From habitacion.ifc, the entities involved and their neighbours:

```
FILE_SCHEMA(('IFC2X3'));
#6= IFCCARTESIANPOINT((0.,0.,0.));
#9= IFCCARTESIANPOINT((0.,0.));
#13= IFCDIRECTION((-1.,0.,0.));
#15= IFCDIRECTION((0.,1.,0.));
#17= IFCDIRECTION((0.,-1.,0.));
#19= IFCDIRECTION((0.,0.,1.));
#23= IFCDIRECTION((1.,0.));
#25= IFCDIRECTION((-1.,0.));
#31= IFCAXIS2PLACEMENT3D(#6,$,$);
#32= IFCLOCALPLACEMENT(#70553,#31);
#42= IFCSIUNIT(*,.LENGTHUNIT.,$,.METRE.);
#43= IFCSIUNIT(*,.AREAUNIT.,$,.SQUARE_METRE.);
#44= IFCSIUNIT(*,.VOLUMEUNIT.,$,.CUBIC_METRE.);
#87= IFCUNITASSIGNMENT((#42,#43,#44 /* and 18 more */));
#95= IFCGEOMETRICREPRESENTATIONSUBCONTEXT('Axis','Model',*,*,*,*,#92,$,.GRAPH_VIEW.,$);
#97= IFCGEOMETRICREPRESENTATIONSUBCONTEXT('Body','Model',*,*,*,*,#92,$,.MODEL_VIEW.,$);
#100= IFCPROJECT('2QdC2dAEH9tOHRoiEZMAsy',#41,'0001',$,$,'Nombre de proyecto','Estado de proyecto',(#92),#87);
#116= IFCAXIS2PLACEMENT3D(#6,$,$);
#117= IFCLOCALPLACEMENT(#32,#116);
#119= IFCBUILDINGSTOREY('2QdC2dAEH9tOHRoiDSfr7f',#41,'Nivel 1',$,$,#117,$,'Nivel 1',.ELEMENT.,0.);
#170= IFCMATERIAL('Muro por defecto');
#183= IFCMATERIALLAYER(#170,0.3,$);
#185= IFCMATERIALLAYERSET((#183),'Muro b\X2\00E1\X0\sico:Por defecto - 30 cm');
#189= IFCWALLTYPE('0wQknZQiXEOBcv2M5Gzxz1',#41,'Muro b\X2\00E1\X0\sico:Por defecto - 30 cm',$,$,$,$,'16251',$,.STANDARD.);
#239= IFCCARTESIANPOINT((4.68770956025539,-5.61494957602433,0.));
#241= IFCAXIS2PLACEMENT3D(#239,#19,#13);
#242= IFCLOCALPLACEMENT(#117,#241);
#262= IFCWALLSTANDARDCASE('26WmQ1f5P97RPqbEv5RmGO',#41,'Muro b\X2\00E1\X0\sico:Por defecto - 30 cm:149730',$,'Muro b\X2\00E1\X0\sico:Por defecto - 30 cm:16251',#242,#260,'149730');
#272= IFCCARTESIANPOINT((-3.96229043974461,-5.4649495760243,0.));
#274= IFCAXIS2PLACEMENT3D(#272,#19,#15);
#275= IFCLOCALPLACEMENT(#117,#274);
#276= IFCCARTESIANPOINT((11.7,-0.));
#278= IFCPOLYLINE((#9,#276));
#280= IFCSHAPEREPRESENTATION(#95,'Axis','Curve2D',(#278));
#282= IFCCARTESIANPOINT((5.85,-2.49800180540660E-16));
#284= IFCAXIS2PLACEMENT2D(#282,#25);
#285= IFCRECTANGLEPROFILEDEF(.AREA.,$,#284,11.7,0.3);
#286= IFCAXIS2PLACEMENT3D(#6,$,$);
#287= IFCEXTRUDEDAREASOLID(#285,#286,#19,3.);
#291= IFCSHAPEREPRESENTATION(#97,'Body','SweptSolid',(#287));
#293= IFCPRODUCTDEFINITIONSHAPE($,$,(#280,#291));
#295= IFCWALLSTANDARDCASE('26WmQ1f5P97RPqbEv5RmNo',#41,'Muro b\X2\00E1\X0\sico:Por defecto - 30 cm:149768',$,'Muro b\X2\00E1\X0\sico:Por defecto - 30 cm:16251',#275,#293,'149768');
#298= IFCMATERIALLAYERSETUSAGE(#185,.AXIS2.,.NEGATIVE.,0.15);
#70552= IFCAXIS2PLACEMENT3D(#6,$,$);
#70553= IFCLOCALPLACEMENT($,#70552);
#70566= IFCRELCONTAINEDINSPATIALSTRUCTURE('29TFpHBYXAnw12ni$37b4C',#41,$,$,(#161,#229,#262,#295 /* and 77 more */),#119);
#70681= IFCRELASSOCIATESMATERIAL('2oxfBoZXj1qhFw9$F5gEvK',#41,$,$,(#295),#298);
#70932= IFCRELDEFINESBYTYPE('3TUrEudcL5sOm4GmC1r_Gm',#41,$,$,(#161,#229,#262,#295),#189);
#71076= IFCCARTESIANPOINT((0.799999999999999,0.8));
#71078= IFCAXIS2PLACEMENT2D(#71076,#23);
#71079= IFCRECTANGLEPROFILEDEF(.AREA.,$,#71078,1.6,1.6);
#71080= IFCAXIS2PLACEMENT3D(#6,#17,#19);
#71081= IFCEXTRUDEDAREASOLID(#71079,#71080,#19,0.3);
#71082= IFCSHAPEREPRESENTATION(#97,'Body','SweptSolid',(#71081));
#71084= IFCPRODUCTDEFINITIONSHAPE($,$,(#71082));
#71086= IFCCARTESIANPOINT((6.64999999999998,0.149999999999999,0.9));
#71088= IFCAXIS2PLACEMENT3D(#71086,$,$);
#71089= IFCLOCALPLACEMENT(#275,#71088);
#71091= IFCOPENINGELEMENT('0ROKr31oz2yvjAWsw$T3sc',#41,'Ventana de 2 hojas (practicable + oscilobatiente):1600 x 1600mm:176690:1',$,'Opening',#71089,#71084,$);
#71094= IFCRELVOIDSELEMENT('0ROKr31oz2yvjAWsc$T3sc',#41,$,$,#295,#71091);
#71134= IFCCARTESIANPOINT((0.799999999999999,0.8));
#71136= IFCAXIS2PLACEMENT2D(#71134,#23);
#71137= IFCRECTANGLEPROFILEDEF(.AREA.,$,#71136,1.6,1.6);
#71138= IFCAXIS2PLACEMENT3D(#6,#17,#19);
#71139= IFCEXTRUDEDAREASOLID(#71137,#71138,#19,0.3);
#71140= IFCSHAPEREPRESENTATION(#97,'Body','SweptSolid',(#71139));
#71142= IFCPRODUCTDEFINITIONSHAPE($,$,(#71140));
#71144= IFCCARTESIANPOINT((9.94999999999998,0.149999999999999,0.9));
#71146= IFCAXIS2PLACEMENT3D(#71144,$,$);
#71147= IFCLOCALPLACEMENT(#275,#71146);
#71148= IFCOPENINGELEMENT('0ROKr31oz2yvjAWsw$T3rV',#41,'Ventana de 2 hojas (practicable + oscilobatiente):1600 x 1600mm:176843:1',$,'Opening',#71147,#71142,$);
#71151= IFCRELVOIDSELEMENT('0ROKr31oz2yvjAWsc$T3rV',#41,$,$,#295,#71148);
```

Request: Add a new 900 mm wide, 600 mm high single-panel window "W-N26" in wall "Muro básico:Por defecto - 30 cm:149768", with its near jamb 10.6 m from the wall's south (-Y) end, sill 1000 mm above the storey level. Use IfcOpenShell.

```python
import numpy as np
import ifcopenshell
import ifcopenshell.api.feature
import ifcopenshell.api.geometry
import ifcopenshell.api.root
import ifcopenshell.api.spatial
import ifcopenshell.api.type
import ifcopenshell.geom
import ifcopenshell.util.element
import ifcopenshell.util.placement
import ifcopenshell.util.representation
import ifcopenshell.util.shape
import ifcopenshell.util.unit

model = ifcopenshell.open("habitacion.ifc")
unit_scale = ifcopenshell.util.unit.calculate_unit_scale(model)
settings = ifcopenshell.geom.settings()


def volume(element):
    """Net volume in cubic metres, openings subtracted."""
    shape = ifcopenshell.geom.create_shape(settings, element)
    return ifcopenshell.util.shape.get_volume(shape.geometry)


wall = model.by_guid("26WmQ1f5P97RPqbEv5RmNo")
storey = ifcopenshell.util.element.get_container(wall, ifc_class="IfcBuildingStorey")
context = ifcopenshell.util.representation.get_context(model, "Model", "Body", "MODEL_VIEW")
before = volume(wall)

width, height, from_end, sill = 0.9, 0.6, 10.6, 1  # metres

# The wall runs along its own X axis, and the end named is its -X end.
wall_shape = ifcopenshell.geom.create_shape(settings, wall)
x, y, z = ifcopenshell.util.shape.get_vertices(wall_shape.geometry).T
start = x.min() + from_end
face, thickness = float(y.min()), float(y.max() - y.min())
wall_matrix = ifcopenshell.util.placement.get_local_placement(wall.ObjectPlacement)
level = ifcopenshell.util.placement.get_local_placement(storey.ObjectPlacement)[2, 3]


def in_wall(x, y):
    """Placement at x, y metres in the wall's axes, at sill height."""
    matrix = wall_matrix.copy()
    matrix[:, 3] = wall_matrix @ np.array([x / unit_scale, y / unit_scale, 0.0, 1.0])
    matrix[2, 3] = level + sill / unit_scale
    return matrix


# Opening: a box that overshoots both wall faces by 50 mm.
opening = ifcopenshell.api.root.create_entity(model, ifc_class="IfcOpeningElement")
box = ifcopenshell.api.geometry.add_wall_representation(
    model, context=context, length=width, height=height, thickness=thickness + 0.1
)
ifcopenshell.api.geometry.assign_representation(model, product=opening, representation=box)
ifcopenshell.api.geometry.edit_object_placement(model, product=opening, matrix=in_wall(start, face - 0.05), is_si=False)
ifcopenshell.api.feature.add_feature(model, feature=opening, element=wall)

window = ifcopenshell.api.root.create_entity(model, ifc_class="IfcWindow", name="W-N26")
window.OverallWidth, window.OverallHeight = width / unit_scale, height / unit_scale
body = ifcopenshell.api.geometry.add_window_representation(
    model,
    context=context,
    overall_width=window.OverallWidth,
    overall_height=window.OverallHeight,
    partition_type="SINGLE_PANEL",
)
ifcopenshell.api.geometry.assign_representation(model, product=window, representation=body)
ifcopenshell.api.spatial.assign_container(model, products=[window], relating_structure=storey)
fills = ifcopenshell.api.feature.add_filling(model, opening=opening, element=window)
fills.OwnerHistory = window.OwnerHistory  # required in IFC2X3

# IFC2X3 keeps the operation on the window style.
style = ifcopenshell.api.root.create_entity(model, ifc_class="IfcWindowStyle", name="W-N26")
style.OperationType, style.ConstructionType = "SINGLE_PANEL", "NOTDEFINED"
style.ParameterTakesPrecedence = style.Sizeable = False
ifcopenshell.api.type.assign_type(model, related_objects=[window], relating_type=style)

# Centre the window in the wall's thickness.
ifcopenshell.api.geometry.edit_object_placement(model, product=window, matrix=in_wall(start, face), is_si=False)
window_shape = ifcopenshell.geom.create_shape(settings, window)
depth = ifcopenshell.util.shape.get_vertices(window_shape.geometry)[:, 1]
offset = face + thickness / 2 - (depth.min() + depth.max()) / 2
ifcopenshell.api.geometry.edit_object_placement(model, product=window, matrix=in_wall(start, offset), is_si=False)

after = volume(wall)

print(f"wall volume {before:.3f} -> {after:.3f} m3")

model.write("habitacion_v2.ifc")
```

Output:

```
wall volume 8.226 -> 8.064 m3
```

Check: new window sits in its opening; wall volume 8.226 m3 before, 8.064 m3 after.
